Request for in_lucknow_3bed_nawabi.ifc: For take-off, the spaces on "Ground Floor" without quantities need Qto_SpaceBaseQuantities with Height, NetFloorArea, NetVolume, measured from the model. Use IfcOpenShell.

First a look at what the model holds.

```python
import ifcopenshell
import ifcopenshell.util.element
import ifcopenshell.util.unit

model = ifcopenshell.open("in_lucknow_3bed_nawabi.ifc")
print(model.schema)
for unit_type in ("LENGTHUNIT", "AREAUNIT", "VOLUMEUNIT"):
    print(unit_type, ifcopenshell.util.unit.calculate_unit_scale(model, unit_type))
storey = next(s for s in model.by_type("IfcBuildingStorey") if s.Name == "Ground Floor")
spaces = [e for e in ifcopenshell.util.element.get_decomposition(storey) if e.is_a("IfcSpace")]
for e in sorted(spaces, key=lambda e: e.id()):
    print(e.id(), e.is_a(), e.Name, list(ifcopenshell.util.element.get_psets(e, qtos_only=True)), sep=" | ")
```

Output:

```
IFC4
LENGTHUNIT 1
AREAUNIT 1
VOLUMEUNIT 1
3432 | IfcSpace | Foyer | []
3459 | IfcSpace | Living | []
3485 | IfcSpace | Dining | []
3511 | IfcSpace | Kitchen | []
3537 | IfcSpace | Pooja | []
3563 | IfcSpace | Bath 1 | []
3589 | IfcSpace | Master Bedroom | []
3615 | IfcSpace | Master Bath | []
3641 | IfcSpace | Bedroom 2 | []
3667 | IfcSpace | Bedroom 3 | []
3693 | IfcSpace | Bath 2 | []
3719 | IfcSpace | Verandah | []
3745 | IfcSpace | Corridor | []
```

```python
import ifcopenshell
import ifcopenshell.api.pset
import ifcopenshell.geom
import ifcopenshell.util.element
import ifcopenshell.util.shape
import ifcopenshell.util.unit

model = ifcopenshell.open("in_lucknow_3bed_nawabi.ifc")
unit_scale = ifcopenshell.util.unit.calculate_unit_scale(model)
area_scale = ifcopenshell.util.unit.calculate_unit_scale(model, "AREAUNIT")
volume_scale = ifcopenshell.util.unit.calculate_unit_scale(model, "VOLUMEUNIT")
settings = ifcopenshell.geom.settings()

storey = next(s for s in model.by_type("IfcBuildingStorey") if s.Name == "Ground Floor")
spaces = [e for e in ifcopenshell.util.element.get_decomposition(storey) if e.is_a("IfcSpace")]

for e in sorted(spaces, key=lambda e: e.id()):
    if ifcopenshell.util.element.get_psets(e, qtos_only=True, should_inherit=False):
        continue
    # Geometry comes back in metres, in the element's own axes.
    shape = ifcopenshell.geom.create_shape(settings, e)
    values = {
        "Height": ifcopenshell.util.shape.get_z(shape.geometry) / unit_scale,
        "NetFloorArea": ifcopenshell.util.shape.get_footprint_area(shape.geometry) / area_scale,
        "NetVolume": ifcopenshell.util.shape.get_volume(shape.geometry) / volume_scale,
    }
    qto = ifcopenshell.api.pset.add_qto(model, product=e, name="Qto_SpaceBaseQuantities")
    ifcopenshell.api.pset.edit_qto(model, qto=qto, properties=values)
    print(e.id(), {k: round(v, 3) for k, v in values.items()})

model.write("in_lucknow_3bed_nawabi_updated.ifc")
```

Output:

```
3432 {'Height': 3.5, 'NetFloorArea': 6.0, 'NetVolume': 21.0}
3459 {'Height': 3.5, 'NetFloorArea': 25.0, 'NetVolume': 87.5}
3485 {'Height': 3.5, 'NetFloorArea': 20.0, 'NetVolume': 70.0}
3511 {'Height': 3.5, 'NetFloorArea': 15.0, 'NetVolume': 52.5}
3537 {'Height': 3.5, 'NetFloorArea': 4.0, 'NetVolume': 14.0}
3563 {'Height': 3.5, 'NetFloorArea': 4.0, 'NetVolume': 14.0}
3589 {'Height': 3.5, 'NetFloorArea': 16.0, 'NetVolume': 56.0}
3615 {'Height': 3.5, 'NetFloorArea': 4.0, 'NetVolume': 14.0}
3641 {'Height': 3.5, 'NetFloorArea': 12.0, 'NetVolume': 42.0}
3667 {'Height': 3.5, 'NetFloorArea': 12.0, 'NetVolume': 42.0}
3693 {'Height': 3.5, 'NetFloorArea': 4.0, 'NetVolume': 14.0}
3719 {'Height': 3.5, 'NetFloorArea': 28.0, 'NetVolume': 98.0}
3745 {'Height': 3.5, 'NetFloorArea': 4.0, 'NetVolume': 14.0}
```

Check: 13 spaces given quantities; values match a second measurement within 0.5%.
